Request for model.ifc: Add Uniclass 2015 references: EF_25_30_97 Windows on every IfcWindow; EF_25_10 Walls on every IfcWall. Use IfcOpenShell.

First a look at what the model holds.

```python
import ifcopenshell

model = ifcopenshell.open("model.ifc")
print(model.schema)
print("classifications:", [c.Name for c in model.by_type("IfcClassification")])
for ifc_class in ("IfcDoor", "IfcRoof", "IfcStair", "IfcWall", "IfcWindow"):
    print(ifc_class, len(model.by_type(ifc_class)))
```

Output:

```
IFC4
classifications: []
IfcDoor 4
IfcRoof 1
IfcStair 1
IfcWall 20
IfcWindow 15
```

```python
import ifcopenshell
import ifcopenshell.api.classification

model = ifcopenshell.open("model.ifc")

system = ifcopenshell.api.classification.add_classification(model, classification="Uniclass 2015")

codes = {
    "IfcWindow": ("EF_25_30_97", "Windows"),
    "IfcWall": ("EF_25_10", "Walls"),
}
for ifc_class, (code, name) in codes.items():
    products = model.by_type(ifc_class)
    ifcopenshell.api.classification.add_reference(
        model, products=products, classification=system, identification=code, name=name
    )
    print(code, len(products))

model.write("model_rev.ifc")
```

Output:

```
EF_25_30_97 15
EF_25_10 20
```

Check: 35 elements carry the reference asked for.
